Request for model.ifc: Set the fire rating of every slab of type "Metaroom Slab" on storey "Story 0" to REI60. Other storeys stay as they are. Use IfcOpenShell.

First a look at what the model holds.

```python
import ifcopenshell
import ifcopenshell.util.element

model = ifcopenshell.open("model.ifc")
print(model.schema)
storey = next(s for s in model.by_type("IfcBuildingStorey") if s.Name == "Story 0")
slabs = [e for e in ifcopenshell.util.element.get_decomposition(storey) if e.is_a("IfcSlab")]
seen = {}
for e in slabs:
    element_type = ifcopenshell.util.element.get_type(e)
    key = (element_type.Name if element_type != e and element_type else None, ifcopenshell.util.element.get_pset(e, "Pset_SlabCommon", "FireRating"))
    seen[key] = seen.get(key, 0) + 1
for (name, value), count in sorted(seen.items(), key=str):
    print(count, "x", name, "|", value)
```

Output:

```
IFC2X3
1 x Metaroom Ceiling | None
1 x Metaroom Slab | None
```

```python
import ifcopenshell
import ifcopenshell.api.pset
import ifcopenshell.util.element

model = ifcopenshell.open("model.ifc")

storey = next(s for s in model.by_type("IfcBuildingStorey") if s.Name == "Story 0")
slabs = [e for e in ifcopenshell.util.element.get_decomposition(storey) if e.is_a("IfcSlab")]

count = 0
for e in slabs:
    element_type = ifcopenshell.util.element.get_type(e)
    if element_type in (None, e) or element_type.Name != "Metaroom Slab":
        continue
    # add_pset returns the element's existing set when there is one.
    pset = ifcopenshell.api.pset.add_pset(model, product=e, name="Pset_SlabCommon")
    ifcopenshell.api.pset.edit_pset(model, pset=pset, properties={"FireRating": "REI60"})
    count += 1

print(count, "slabs updated")

model.write("model_edited.ifc")
```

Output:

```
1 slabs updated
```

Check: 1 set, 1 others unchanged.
